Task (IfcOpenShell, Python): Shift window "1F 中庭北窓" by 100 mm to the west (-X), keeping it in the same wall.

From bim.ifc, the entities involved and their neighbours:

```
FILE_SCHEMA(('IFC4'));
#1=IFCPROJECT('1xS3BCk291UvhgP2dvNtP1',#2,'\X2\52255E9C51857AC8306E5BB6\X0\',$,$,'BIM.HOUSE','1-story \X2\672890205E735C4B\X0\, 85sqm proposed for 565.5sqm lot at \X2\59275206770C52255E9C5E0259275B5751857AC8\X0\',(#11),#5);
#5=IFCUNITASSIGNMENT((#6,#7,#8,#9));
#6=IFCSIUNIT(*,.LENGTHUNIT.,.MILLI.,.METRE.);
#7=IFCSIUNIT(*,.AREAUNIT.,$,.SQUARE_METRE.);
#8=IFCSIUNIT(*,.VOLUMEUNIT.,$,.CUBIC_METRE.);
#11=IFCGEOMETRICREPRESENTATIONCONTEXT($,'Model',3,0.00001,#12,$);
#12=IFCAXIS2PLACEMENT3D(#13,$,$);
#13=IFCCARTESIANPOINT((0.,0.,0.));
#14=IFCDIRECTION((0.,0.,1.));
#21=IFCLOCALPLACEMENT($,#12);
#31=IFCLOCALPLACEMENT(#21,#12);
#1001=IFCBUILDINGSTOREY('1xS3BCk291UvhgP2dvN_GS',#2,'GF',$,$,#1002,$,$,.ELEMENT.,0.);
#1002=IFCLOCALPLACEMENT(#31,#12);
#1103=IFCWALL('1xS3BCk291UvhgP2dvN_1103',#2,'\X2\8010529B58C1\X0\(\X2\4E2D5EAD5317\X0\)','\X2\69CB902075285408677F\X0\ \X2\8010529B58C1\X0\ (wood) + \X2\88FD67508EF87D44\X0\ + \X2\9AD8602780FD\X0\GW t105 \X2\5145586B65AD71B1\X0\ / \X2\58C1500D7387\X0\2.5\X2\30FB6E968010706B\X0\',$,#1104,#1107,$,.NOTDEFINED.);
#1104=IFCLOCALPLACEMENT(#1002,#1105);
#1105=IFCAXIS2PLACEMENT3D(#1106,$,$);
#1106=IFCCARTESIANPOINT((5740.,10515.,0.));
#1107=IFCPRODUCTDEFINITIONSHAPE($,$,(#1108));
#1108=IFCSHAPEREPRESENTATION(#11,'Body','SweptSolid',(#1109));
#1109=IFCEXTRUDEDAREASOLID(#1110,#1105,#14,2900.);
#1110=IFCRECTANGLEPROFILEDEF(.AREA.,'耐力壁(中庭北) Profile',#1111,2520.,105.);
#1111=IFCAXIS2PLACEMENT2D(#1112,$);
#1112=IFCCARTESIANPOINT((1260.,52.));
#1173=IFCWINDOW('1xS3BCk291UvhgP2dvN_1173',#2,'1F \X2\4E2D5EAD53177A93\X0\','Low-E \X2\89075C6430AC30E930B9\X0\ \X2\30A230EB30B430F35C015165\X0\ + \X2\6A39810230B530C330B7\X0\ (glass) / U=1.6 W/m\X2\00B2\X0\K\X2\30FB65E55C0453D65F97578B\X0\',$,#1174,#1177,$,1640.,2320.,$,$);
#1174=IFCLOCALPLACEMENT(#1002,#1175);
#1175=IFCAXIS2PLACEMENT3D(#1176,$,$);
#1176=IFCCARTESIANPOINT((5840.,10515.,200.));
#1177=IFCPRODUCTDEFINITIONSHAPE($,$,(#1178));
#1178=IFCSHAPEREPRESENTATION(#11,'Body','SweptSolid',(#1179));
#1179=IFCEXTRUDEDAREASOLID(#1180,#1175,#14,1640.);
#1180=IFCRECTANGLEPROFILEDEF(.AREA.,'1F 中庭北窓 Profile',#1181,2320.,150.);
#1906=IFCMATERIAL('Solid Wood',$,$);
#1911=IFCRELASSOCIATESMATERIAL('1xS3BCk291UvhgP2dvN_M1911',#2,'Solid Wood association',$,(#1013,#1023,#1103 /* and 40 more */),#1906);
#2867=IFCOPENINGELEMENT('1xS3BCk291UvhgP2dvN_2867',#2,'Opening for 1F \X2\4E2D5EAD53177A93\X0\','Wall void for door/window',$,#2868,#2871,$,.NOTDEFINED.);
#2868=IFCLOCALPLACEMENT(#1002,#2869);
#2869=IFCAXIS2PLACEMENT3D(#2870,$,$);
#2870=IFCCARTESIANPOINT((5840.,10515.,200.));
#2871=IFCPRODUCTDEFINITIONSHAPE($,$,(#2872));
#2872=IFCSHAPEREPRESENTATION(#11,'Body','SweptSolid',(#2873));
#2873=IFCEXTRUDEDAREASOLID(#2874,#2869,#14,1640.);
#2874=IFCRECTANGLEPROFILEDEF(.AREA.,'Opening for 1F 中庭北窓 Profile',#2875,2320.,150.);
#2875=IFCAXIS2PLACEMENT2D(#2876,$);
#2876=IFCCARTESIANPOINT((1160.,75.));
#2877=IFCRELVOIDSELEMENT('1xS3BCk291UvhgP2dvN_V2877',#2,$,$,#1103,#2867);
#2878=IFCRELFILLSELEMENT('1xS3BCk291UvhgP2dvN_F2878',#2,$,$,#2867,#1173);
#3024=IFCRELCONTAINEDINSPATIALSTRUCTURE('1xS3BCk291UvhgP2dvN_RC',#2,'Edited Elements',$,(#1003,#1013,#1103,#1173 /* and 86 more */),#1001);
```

```python
import ifcopenshell
import ifcopenshell.api.geometry
import ifcopenshell.util.placement

model = ifcopenshell.open("bim.ifc")

window = model.by_guid("1xS3BCk291UvhgP2dvN_1173")
opening = window.FillsVoids[0].RelatingOpeningElement
wall = opening.VoidsElements[0].RelatingBuildingElement

wall_matrix = ifcopenshell.util.placement.get_local_placement(wall.ObjectPlacement)
shift = wall_matrix[:3, 0] * -100.0
before = ifcopenshell.util.placement.get_local_placement(window.ObjectPlacement)[:3, 3].copy()

# The window is not placed relative to its opening, so move both.
for product in (opening, window):
    matrix = ifcopenshell.util.placement.get_local_placement(product.ObjectPlacement)
    matrix[:3, 3] += shift
    ifcopenshell.api.geometry.edit_object_placement(model, product=product, matrix=matrix, is_si=False)

after = ifcopenshell.util.placement.get_local_placement(window.ObjectPlacement)[:3, 3]
print("window moved by", (after - before).round(3) + 0.0)

model.write("bim_v2.ifc")
```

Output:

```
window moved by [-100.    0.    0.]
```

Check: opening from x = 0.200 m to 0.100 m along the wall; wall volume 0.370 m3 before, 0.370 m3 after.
